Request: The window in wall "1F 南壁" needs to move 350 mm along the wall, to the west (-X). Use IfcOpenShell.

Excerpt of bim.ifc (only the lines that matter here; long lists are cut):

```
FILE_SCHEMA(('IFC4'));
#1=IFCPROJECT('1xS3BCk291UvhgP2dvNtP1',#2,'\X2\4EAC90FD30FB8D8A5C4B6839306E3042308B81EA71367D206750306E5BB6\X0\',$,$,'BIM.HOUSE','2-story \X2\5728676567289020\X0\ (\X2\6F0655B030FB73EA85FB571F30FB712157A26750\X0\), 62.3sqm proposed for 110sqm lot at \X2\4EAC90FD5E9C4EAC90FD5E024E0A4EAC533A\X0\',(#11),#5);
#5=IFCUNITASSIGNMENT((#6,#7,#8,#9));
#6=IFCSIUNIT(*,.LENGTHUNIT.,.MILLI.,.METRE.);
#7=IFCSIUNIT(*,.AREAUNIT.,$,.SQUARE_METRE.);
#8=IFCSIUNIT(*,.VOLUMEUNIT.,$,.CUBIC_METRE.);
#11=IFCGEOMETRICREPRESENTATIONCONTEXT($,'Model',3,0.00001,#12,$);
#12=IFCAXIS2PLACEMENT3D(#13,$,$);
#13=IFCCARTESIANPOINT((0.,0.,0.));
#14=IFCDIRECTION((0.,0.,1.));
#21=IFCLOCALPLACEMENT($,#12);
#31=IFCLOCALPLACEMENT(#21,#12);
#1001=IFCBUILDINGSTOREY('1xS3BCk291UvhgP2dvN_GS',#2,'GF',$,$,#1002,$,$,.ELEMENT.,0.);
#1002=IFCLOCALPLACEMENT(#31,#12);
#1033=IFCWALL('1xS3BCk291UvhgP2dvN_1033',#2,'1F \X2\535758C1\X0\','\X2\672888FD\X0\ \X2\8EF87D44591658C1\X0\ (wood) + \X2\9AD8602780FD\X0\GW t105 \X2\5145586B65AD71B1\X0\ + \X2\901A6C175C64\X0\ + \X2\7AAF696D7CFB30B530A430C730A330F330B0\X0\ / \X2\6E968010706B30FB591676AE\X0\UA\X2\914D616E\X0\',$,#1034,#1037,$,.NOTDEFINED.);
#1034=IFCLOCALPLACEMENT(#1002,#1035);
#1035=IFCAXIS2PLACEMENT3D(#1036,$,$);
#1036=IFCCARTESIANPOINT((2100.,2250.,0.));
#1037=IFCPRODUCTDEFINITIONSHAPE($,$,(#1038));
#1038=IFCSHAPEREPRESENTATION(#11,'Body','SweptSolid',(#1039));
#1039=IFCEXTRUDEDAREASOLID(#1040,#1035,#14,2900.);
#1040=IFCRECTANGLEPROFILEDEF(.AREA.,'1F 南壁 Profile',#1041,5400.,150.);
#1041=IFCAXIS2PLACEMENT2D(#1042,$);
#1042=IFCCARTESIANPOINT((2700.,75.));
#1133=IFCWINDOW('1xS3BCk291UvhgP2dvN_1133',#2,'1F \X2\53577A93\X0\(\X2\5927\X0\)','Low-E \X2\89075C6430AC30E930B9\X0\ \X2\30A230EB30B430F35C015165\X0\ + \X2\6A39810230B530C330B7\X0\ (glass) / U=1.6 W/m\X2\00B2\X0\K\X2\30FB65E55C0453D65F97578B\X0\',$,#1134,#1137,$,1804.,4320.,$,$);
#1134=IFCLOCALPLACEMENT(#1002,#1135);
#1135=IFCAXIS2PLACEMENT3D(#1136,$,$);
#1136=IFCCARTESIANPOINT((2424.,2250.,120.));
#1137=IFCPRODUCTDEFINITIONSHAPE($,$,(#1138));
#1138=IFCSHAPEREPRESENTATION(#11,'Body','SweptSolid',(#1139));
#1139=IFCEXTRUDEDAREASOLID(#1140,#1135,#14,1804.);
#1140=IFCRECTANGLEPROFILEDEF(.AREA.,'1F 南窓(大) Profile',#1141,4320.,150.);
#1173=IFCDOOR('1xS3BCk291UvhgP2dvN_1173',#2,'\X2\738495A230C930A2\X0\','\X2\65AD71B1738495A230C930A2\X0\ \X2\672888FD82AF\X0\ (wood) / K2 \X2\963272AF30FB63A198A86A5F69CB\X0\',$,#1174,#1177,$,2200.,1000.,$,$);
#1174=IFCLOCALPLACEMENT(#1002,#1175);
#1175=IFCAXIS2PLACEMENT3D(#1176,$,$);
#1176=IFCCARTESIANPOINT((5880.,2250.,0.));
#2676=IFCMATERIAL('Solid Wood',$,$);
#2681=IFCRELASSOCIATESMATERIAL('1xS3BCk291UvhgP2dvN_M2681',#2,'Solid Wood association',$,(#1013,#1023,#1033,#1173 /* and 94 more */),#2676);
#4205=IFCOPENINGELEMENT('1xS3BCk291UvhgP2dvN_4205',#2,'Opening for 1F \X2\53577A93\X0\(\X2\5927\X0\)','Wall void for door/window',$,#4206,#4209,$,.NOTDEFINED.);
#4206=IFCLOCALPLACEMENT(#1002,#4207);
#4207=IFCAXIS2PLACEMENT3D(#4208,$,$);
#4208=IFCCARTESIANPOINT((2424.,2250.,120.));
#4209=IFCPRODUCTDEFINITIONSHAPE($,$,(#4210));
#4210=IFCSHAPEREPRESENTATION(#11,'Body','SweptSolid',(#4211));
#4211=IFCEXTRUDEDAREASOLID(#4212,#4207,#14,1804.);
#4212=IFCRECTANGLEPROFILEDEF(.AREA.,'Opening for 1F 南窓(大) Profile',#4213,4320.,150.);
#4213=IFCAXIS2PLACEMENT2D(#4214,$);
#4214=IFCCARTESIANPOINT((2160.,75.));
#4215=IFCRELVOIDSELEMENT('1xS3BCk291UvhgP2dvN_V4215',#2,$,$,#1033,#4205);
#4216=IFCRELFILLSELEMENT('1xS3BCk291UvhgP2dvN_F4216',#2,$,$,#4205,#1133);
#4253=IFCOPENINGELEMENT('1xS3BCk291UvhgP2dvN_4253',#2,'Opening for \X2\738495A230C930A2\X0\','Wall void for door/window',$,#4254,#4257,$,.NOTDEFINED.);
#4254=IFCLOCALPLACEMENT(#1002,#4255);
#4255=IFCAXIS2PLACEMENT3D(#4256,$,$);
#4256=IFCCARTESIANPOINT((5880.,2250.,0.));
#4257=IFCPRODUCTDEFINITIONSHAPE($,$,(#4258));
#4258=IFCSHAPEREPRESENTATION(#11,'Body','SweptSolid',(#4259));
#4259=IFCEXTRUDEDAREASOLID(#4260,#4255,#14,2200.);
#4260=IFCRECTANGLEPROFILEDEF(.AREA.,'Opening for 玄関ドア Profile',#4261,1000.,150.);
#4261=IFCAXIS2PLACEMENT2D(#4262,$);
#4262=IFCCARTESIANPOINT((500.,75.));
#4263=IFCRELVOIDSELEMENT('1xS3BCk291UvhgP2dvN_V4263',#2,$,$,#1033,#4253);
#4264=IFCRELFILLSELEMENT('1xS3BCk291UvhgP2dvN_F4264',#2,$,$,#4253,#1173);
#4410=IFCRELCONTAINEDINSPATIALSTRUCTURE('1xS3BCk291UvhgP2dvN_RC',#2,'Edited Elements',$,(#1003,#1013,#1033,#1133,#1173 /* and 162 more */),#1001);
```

```python
import ifcopenshell
import ifcopenshell.api.geometry
import ifcopenshell.util.placement
import ifcopenshell.util.unit

model = ifcopenshell.open("bim.ifc")
unit_scale = ifcopenshell.util.unit.calculate_unit_scale(model)

window = model.by_guid("1xS3BCk291UvhgP2dvN_1133")
opening = window.FillsVoids[0].RelatingOpeningElement
wall = opening.VoidsElements[0].RelatingBuildingElement

wall_matrix = ifcopenshell.util.placement.get_local_placement(wall.ObjectPlacement)
shift = wall_matrix[:3, 0] * -0.35 / unit_scale
before = ifcopenshell.util.placement.get_local_placement(window.ObjectPlacement)[:3, 3].copy()

# The window is not placed relative to its opening, so move both.
for product in (opening, window):
    matrix = ifcopenshell.util.placement.get_local_placement(product.ObjectPlacement)
    matrix[:3, 3] += shift
    ifcopenshell.api.geometry.edit_object_placement(model, product=product, matrix=matrix, is_si=False)

after = ifcopenshell.util.placement.get_local_placement(window.ObjectPlacement)[:3, 3]
print("window moved by", (after - before).round(3) + 0.0)

model.write("bim_rev.ifc")
```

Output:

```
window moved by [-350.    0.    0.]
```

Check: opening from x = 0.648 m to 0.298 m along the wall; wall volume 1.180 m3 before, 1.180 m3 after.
